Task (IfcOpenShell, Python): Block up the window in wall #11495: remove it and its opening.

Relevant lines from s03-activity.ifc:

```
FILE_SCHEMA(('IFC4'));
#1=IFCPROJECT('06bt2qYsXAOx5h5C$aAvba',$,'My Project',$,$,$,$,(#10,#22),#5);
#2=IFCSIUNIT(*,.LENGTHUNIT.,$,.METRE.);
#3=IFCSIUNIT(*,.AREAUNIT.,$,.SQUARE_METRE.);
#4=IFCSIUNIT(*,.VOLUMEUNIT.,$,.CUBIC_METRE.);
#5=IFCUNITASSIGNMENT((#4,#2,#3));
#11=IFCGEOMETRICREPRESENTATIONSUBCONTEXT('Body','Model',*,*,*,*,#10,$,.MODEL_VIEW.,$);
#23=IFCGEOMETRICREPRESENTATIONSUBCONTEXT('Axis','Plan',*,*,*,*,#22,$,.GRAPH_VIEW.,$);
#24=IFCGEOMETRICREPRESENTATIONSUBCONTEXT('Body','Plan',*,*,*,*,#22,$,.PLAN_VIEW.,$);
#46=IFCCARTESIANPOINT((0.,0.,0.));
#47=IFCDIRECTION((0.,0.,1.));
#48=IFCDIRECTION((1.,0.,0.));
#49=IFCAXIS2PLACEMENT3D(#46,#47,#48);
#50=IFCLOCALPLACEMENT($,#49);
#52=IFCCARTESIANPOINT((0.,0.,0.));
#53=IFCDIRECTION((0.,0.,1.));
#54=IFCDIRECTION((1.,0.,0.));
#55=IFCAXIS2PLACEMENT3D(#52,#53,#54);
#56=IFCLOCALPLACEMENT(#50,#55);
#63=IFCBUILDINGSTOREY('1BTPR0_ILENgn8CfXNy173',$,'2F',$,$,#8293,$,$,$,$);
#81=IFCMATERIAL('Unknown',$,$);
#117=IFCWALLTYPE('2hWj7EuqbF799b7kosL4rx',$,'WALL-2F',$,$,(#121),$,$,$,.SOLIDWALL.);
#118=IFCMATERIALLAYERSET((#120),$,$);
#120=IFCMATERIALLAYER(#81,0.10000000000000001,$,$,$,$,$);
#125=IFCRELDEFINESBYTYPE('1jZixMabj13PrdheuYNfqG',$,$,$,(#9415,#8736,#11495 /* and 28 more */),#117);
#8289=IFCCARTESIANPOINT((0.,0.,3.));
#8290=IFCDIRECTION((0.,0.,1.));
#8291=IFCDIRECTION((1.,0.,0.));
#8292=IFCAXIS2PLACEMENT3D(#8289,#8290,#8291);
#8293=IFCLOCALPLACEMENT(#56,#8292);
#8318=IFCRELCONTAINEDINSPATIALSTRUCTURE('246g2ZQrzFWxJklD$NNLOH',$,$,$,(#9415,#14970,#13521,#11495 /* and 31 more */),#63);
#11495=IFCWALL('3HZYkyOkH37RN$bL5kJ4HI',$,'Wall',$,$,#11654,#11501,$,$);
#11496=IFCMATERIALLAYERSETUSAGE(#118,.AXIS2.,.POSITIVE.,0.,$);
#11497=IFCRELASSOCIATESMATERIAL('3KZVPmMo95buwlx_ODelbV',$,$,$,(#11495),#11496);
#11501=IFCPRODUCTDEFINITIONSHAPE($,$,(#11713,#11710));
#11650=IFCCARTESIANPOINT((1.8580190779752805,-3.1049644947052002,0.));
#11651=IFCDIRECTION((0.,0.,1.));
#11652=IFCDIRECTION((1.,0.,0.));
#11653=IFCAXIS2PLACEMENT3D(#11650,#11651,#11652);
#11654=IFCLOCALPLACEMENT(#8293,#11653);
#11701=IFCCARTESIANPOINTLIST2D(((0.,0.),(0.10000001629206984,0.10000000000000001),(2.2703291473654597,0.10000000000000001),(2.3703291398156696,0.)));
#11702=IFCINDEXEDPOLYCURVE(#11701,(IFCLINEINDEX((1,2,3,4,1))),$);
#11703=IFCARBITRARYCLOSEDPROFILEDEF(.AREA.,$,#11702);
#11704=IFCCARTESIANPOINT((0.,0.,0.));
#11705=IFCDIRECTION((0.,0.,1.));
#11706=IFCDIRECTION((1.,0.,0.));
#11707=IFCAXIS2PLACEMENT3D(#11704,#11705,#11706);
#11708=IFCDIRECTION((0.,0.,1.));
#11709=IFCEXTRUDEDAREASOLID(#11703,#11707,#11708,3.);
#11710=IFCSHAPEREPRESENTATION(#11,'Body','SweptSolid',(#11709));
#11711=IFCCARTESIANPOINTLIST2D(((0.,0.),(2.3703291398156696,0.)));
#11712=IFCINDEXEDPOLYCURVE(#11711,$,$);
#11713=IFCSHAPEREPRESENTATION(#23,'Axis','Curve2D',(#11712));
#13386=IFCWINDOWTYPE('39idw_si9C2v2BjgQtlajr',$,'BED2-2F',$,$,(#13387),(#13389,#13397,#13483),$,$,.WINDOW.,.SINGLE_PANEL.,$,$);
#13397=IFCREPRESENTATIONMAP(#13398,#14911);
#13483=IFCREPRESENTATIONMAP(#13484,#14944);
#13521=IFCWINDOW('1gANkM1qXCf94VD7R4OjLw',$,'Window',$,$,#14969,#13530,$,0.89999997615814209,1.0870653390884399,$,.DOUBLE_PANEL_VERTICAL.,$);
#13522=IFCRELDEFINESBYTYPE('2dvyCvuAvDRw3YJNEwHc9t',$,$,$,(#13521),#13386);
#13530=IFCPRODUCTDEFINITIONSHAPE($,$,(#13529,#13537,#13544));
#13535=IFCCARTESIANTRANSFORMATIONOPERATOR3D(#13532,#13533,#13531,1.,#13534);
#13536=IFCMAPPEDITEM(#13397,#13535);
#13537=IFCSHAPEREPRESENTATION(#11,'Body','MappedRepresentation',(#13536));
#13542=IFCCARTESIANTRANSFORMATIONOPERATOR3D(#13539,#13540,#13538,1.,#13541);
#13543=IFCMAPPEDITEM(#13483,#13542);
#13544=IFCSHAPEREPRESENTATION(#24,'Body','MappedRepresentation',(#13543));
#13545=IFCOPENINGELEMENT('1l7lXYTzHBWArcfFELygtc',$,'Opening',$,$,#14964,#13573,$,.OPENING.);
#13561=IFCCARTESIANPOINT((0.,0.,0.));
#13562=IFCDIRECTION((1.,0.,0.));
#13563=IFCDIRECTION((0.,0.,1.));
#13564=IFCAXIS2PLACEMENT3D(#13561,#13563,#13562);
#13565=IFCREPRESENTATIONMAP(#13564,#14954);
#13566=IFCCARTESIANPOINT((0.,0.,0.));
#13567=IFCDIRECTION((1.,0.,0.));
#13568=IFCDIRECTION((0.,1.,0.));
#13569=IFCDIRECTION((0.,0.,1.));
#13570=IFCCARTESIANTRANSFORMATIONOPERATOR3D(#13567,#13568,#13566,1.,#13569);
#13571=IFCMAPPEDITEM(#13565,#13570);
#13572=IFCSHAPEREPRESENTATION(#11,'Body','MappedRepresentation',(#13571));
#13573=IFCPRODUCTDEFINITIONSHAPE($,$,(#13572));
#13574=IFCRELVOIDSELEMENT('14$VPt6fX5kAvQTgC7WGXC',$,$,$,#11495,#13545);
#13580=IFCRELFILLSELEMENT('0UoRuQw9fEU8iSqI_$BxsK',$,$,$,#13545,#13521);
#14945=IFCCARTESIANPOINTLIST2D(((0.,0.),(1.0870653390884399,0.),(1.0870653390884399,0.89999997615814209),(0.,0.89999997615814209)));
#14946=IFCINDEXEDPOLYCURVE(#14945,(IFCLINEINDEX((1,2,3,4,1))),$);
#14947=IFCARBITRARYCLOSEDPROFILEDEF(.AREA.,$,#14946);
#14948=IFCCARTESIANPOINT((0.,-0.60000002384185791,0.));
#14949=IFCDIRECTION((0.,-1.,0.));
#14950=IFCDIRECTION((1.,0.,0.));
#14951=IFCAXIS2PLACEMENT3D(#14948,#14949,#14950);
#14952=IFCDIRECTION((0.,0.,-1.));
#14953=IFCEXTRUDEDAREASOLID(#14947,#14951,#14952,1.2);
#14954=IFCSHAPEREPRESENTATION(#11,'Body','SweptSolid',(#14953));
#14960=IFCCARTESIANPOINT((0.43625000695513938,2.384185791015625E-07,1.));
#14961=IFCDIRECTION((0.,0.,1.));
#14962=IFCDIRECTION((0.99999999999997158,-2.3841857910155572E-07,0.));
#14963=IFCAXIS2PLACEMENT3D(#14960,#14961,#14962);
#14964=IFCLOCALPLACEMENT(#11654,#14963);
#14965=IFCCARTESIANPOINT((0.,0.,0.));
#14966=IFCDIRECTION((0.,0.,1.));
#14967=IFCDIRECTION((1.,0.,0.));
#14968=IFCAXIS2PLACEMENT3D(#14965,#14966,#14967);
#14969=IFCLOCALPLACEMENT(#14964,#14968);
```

```python
import ifcopenshell
import ifcopenshell.api.feature
import ifcopenshell.api.root
import ifcopenshell.geom
import ifcopenshell.util.shape

model = ifcopenshell.open("s03-activity.ifc")
settings = ifcopenshell.geom.settings()


def volume(element):
    """Net volume in cubic metres, openings subtracted."""
    shape = ifcopenshell.geom.create_shape(settings, element)
    return ifcopenshell.util.shape.get_volume(shape.geometry)


window = model.by_guid("1gANkM1qXCf94VD7R4OjLw")
opening = window.FillsVoids[0].RelatingOpeningElement
wall = opening.VoidsElements[0].RelatingBuildingElement
before = volume(wall)

ifcopenshell.api.root.remove_product(model, product=window)
ifcopenshell.api.feature.remove_feature(model, feature=opening)

after = volume(wall)

print(f"wall volume {before:.3f} -> {after:.3f} m3")

model.write("s03-activity_rev.ifc")
```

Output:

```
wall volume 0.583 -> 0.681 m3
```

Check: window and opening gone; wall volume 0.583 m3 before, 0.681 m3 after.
